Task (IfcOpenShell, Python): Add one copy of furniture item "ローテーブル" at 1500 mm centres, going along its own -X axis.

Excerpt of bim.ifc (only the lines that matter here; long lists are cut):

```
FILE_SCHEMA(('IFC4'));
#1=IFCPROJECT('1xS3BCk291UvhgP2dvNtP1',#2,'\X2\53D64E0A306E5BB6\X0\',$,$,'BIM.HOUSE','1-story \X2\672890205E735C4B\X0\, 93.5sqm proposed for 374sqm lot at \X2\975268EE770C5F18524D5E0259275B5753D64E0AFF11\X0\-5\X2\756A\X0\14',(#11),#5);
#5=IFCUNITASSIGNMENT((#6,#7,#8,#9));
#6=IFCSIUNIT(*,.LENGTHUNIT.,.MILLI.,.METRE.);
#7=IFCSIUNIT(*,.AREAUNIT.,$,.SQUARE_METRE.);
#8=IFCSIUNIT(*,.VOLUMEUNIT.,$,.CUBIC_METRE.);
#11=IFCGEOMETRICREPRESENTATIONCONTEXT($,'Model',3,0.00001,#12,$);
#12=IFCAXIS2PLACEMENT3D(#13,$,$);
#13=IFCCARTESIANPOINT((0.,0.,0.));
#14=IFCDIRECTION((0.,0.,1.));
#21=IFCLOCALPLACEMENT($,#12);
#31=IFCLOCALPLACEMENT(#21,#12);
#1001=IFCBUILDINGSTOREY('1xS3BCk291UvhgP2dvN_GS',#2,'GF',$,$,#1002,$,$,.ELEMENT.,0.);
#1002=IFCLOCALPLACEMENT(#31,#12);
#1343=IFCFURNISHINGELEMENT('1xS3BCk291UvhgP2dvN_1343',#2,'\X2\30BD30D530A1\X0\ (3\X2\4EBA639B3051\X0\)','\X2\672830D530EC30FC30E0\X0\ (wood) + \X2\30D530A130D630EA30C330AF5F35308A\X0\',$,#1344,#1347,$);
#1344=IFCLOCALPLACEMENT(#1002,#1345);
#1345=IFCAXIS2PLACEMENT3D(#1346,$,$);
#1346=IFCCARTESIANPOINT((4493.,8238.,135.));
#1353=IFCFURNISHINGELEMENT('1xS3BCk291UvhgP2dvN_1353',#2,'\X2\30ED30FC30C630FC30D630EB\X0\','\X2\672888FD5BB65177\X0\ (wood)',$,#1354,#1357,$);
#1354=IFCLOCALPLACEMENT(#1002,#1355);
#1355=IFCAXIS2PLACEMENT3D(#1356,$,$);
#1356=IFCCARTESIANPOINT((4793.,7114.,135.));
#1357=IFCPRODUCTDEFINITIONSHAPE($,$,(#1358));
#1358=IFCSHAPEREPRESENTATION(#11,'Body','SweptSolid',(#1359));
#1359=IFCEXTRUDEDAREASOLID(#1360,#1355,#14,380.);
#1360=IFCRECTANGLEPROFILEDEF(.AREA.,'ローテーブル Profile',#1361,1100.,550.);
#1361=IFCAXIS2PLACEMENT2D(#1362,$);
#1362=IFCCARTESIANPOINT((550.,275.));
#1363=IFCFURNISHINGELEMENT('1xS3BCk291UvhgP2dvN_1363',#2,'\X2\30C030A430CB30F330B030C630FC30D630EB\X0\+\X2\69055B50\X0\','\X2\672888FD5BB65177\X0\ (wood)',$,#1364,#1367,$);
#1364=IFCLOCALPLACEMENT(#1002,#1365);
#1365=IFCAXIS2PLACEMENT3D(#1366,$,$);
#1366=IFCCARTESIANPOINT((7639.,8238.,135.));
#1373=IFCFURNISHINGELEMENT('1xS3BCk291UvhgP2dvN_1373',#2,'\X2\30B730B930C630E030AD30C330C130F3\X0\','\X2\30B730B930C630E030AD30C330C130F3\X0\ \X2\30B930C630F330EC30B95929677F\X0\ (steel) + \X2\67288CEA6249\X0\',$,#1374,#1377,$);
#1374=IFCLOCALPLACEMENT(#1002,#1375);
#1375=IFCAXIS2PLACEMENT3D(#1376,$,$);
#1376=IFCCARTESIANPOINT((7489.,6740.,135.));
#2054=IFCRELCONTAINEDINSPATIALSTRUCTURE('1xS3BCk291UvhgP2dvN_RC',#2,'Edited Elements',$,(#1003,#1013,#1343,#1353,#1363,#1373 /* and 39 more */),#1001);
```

```python
import ifcopenshell
import ifcopenshell.api.geometry
import ifcopenshell.api.root
import ifcopenshell.util.element
import ifcopenshell.util.placement
import ifcopenshell.util.unit

model = ifcopenshell.open("bim.ifc")
unit_scale = ifcopenshell.util.unit.calculate_unit_scale(model)


def reuse_history(source, copy):
    """copy_class also copies each property set's owner history, people and application; keep the originals."""
    for rel in copy.IsDefinedBy:
        if rel.is_a("IfcRelDefinesByProperties") and (history := rel.RelatingPropertyDefinition.OwnerHistory):
            rel.RelatingPropertyDefinition.OwnerHistory = source.OwnerHistory
            ifcopenshell.util.element.remove_deep2(model, history)


source = model.by_guid("1xS3BCk291UvhgP2dvN_1353")
base = ifcopenshell.util.placement.get_local_placement(source.ObjectPlacement)
step = -base[:3, 0] * 1.5 / unit_scale

for i in range(1, 2):
    copy = ifcopenshell.api.root.copy_class(model, product=source)
    copy.Representation = ifcopenshell.util.element.copy_deep(
        model, source.Representation, exclude=["IfcGeometricRepresentationContext", "IfcRepresentationMap"]
    )
    reuse_history(source, copy)
    matrix = base.copy()
    matrix[:3, 3] += i * step
    print("added at", matrix[:3, 3].round(3) + 0.0)
    ifcopenshell.api.geometry.edit_object_placement(model, product=copy, matrix=matrix, is_si=False)

model.write("bim_updated.ifc")
```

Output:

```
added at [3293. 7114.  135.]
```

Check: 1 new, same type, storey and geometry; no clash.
